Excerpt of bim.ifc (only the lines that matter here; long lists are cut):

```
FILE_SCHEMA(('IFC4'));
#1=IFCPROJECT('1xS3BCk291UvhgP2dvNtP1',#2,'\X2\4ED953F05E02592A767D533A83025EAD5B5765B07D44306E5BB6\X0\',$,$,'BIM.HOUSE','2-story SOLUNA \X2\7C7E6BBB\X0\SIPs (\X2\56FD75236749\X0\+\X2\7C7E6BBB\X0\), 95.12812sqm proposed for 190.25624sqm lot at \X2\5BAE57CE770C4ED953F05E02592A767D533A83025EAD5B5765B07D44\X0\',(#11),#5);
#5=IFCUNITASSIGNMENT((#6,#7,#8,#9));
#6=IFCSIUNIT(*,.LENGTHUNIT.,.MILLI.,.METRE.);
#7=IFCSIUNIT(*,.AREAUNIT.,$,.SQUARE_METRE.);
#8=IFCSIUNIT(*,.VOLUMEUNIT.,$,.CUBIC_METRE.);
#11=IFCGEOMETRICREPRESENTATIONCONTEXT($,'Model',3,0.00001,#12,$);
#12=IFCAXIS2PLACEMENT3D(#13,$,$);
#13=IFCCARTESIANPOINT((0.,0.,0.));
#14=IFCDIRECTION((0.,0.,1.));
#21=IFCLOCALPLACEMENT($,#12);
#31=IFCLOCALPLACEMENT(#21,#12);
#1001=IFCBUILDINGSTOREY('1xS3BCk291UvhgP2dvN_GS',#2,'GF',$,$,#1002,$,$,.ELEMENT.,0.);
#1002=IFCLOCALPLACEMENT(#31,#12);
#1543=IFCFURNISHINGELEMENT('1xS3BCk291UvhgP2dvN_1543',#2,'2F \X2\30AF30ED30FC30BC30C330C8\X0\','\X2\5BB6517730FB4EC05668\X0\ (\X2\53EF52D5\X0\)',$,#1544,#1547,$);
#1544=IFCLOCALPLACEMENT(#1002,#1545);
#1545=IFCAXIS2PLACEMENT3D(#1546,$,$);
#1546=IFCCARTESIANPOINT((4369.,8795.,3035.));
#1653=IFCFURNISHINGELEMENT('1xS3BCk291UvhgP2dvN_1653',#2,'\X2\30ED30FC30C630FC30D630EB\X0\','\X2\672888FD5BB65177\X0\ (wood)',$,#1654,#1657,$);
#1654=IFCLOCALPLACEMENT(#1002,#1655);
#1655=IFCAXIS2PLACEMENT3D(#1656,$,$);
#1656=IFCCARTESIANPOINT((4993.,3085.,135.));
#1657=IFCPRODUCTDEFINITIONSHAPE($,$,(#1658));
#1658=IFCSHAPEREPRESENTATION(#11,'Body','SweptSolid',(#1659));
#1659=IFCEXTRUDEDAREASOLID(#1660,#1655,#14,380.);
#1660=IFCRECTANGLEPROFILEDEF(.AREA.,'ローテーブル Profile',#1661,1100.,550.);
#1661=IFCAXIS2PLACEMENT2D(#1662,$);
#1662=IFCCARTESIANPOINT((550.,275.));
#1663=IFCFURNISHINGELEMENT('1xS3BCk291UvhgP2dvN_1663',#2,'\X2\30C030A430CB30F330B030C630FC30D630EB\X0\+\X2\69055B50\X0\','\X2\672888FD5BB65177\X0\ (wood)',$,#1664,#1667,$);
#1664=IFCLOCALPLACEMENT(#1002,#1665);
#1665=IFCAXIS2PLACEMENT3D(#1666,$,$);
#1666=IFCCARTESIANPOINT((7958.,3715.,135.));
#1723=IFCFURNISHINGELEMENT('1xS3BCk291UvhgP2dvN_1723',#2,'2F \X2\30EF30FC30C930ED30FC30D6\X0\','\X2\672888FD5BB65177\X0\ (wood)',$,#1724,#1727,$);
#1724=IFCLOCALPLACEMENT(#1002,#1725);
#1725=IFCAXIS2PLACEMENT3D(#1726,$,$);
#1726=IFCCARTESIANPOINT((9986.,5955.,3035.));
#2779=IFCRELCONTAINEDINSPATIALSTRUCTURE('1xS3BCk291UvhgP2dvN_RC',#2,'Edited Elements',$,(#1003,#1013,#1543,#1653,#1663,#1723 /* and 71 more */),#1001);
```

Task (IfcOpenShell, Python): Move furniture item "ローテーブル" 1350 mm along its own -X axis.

```python
import ifcopenshell
import ifcopenshell.api.geometry
import ifcopenshell.util.placement
import ifcopenshell.util.unit

model = ifcopenshell.open("bim.ifc")
unit_scale = ifcopenshell.util.unit.calculate_unit_scale(model)

item = model.by_guid("1xS3BCk291UvhgP2dvN_1653")
matrix = ifcopenshell.util.placement.get_local_placement(item.ObjectPlacement)
matrix[:3, 3] -= matrix[:3, 0] * 1.35 / unit_scale
ifcopenshell.api.geometry.edit_object_placement(model, product=item, matrix=matrix, is_si=False)

print(ifcopenshell.util.placement.get_local_placement(item.ObjectPlacement).round(3) + 0.0)

model.write("bim_updated.ifc")
```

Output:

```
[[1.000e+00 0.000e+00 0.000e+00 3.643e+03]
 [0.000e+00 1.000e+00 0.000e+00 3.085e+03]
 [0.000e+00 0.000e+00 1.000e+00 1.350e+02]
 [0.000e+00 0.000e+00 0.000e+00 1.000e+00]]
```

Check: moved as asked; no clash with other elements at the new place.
